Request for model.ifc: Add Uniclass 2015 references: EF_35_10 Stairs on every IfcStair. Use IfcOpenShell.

First a look at what the model holds.

```python
import ifcopenshell

model = ifcopenshell.open("model.ifc")
print(model.schema)
print("classifications:", [c.Name for c in model.by_type("IfcClassification")])
for ifc_class in ("IfcDoor", "IfcRoof", "IfcStair", "IfcWall", "IfcWindow"):
    print(ifc_class, len(model.by_type(ifc_class)))
```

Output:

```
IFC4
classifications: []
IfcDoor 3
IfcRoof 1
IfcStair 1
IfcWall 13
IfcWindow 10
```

```python
import ifcopenshell
import ifcopenshell.api.classification

model = ifcopenshell.open("model.ifc")

system = ifcopenshell.api.classification.add_classification(model, classification="Uniclass 2015")

codes = {
    "IfcStair": ("EF_35_10", "Stairs"),
}
for ifc_class, (code, name) in codes.items():
    products = model.by_type(ifc_class)
    ifcopenshell.api.classification.add_reference(
        model, products=products, classification=system, identification=code, name=name
    )
    print(code, len(products))

model.write("model-out.ifc")
```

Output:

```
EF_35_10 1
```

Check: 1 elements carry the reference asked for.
